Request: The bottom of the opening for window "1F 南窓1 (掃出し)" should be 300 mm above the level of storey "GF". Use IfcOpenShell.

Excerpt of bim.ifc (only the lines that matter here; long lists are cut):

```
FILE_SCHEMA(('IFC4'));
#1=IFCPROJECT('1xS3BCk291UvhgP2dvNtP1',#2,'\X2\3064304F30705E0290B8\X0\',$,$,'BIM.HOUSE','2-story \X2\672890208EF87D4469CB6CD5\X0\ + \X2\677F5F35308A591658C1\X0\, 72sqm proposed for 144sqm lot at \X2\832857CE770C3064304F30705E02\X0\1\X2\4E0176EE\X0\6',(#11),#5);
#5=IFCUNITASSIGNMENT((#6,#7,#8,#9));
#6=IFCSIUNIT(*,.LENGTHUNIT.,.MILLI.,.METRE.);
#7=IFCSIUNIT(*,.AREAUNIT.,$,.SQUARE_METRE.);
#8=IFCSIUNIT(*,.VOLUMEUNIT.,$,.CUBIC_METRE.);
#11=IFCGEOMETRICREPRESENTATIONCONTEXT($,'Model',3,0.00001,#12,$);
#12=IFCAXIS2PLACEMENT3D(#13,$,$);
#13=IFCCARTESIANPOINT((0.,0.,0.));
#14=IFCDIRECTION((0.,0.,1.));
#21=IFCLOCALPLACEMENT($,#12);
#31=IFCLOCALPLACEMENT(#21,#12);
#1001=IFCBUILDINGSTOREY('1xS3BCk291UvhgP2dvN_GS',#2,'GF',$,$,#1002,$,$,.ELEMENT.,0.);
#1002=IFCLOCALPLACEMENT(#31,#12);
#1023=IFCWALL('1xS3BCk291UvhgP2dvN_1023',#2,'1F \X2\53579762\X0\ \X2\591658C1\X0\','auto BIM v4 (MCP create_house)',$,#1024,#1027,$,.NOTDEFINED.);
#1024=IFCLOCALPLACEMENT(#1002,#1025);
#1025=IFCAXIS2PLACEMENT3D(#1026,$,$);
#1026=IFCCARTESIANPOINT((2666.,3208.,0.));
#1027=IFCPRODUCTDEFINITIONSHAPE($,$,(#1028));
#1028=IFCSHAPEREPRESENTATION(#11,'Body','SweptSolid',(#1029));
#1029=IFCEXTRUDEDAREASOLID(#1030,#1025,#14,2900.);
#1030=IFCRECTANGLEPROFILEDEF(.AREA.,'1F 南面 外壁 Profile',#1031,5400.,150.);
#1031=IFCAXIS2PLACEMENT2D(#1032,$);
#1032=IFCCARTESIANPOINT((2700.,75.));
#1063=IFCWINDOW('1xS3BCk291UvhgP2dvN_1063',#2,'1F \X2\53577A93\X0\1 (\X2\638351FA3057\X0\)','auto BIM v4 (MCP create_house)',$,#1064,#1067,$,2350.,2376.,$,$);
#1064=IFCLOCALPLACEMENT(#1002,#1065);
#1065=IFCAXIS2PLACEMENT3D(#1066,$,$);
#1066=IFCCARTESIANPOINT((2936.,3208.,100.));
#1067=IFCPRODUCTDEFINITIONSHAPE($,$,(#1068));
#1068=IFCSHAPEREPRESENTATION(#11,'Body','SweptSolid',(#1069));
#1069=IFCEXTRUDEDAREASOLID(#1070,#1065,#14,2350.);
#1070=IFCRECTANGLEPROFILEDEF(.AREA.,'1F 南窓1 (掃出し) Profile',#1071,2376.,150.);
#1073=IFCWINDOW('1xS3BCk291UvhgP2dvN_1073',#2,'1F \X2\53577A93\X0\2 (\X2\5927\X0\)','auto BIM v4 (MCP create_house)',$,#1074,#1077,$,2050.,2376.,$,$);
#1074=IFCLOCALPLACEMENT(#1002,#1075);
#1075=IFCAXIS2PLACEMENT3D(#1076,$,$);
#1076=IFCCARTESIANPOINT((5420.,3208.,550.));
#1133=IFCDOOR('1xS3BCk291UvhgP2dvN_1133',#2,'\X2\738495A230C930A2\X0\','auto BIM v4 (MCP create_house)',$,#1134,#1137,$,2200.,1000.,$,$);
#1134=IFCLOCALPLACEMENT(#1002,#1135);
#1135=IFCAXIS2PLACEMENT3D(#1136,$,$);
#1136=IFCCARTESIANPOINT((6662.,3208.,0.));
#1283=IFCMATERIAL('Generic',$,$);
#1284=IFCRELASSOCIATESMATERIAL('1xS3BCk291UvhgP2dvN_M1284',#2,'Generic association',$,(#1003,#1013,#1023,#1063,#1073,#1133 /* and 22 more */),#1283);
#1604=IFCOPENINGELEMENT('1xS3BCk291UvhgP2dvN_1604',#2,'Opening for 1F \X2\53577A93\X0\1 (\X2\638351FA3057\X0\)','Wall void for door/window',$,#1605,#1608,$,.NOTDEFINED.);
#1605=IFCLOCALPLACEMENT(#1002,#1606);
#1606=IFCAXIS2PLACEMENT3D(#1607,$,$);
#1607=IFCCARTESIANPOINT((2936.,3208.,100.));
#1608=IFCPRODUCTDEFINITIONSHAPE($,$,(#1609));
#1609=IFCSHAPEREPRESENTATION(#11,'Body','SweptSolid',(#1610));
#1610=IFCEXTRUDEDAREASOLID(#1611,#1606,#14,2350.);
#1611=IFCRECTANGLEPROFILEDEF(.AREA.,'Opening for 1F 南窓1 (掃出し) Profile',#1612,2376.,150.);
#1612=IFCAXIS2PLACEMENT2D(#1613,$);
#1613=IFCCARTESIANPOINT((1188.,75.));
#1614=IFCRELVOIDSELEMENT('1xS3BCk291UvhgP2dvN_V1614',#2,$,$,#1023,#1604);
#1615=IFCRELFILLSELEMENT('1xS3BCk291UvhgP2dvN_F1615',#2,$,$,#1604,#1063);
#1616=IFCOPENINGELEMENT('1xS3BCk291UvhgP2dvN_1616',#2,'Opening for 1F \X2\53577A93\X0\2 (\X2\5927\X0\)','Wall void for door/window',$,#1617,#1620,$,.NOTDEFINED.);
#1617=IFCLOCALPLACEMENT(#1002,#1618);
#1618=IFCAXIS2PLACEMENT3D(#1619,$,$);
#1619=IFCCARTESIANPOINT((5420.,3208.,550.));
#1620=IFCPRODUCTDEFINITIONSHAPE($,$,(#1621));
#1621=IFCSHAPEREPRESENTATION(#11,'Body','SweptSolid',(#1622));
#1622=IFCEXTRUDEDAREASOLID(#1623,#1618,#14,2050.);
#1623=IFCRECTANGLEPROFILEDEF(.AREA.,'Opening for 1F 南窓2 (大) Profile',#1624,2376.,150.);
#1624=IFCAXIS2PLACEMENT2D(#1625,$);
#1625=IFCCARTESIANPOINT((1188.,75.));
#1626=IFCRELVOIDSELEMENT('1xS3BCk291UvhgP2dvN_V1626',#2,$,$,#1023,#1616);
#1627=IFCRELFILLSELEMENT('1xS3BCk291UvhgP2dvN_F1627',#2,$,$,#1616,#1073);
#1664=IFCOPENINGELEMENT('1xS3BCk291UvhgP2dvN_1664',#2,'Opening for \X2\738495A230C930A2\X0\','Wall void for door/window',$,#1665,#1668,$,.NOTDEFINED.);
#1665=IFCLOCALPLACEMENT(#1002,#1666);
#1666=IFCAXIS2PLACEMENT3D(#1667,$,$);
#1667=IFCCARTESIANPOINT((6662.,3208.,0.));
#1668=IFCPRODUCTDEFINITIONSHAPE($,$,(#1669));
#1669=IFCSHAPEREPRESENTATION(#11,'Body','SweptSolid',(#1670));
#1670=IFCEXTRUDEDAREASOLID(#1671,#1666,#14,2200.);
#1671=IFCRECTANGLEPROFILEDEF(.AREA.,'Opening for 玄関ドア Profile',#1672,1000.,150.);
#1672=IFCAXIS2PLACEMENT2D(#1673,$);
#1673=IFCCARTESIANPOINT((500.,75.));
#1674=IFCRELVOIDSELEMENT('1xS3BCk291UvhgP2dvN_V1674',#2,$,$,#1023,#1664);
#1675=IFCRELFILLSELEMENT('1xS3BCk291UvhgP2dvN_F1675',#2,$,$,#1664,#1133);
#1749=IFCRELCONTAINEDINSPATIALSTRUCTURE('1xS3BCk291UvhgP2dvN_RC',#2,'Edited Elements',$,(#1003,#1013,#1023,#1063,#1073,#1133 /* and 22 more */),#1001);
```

```python
import numpy as np
import ifcopenshell
import ifcopenshell.api.geometry
import ifcopenshell.geom
import ifcopenshell.util.element
import ifcopenshell.util.placement
import ifcopenshell.util.shape
import ifcopenshell.util.unit

model = ifcopenshell.open("bim.ifc")
unit_scale = ifcopenshell.util.unit.calculate_unit_scale(model)

window = model.by_guid("1xS3BCk291UvhgP2dvN_1063")
opening = window.FillsVoids[0].RelatingOpeningElement
storey = ifcopenshell.util.element.get_container(window, ifc_class="IfcBuildingStorey")
level = ifcopenshell.util.placement.get_local_placement(storey.ObjectPlacement)[2, 3]

# The opening's origin need not be at the sill, so measure its lowest point.
shape = ifcopenshell.geom.create_shape(ifcopenshell.geom.settings(), opening)
bottom = ifcopenshell.util.shape.get_shape_bottom_elevation(shape, shape.geometry) / unit_scale
dz = level + 0.3 / unit_scale - bottom

shift = np.array([0.0, 0.0, dz])
# The window is not placed relative to its opening, so move both.
for product in (opening, window):
    matrix = ifcopenshell.util.placement.get_local_placement(product.ObjectPlacement)
    matrix[:3, 3] += shift
    ifcopenshell.api.geometry.edit_object_placement(model, product=product, matrix=matrix, is_si=False)

print(f"moved by {dz * unit_scale:+.3f} m")

model.write("bim_v2.ifc")
```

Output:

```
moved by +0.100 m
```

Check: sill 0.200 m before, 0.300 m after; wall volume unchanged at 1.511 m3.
